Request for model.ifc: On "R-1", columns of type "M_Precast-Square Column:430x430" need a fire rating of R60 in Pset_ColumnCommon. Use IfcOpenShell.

First a look at what the model holds.

```python
import ifcopenshell
import ifcopenshell.util.element

model = ifcopenshell.open("model.ifc")
print(model.schema)
storey = next(s for s in model.by_type("IfcBuildingStorey") if s.Name == "R-1")
columns = [e for e in ifcopenshell.util.element.get_decomposition(storey) if e.is_a("IfcColumn")]
seen = {}
for e in columns:
    element_type = ifcopenshell.util.element.get_type(e)
    key = (element_type.Name if element_type != e and element_type else None, ifcopenshell.util.element.get_pset(e, "Pset_ColumnCommon", "FireRating"))
    seen[key] = seen.get(key, 0) + 1
for (name, value), count in sorted(seen.items(), key=str):
    print(count, "x", name, "|", value)
```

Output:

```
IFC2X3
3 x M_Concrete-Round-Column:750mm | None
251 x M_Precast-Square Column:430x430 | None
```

```python
import ifcopenshell
import ifcopenshell.api.pset
import ifcopenshell.util.element

model = ifcopenshell.open("model.ifc")

storey = next(s for s in model.by_type("IfcBuildingStorey") if s.Name == "R-1")
columns = [e for e in ifcopenshell.util.element.get_decomposition(storey) if e.is_a("IfcColumn")]

count = 0
for e in columns:
    element_type = ifcopenshell.util.element.get_type(e)
    if element_type in (None, e) or element_type.Name != "M_Precast-Square Column:430x430":
        continue
    # add_pset returns the element's existing set when there is one.
    pset = ifcopenshell.api.pset.add_pset(model, product=e, name="Pset_ColumnCommon")
    ifcopenshell.api.pset.edit_pset(model, pset=pset, properties={"FireRating": "R60"})
    count += 1

print(count, "columns updated")

model.write("model_updated.ifc")
```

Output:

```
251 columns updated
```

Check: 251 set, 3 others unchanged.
